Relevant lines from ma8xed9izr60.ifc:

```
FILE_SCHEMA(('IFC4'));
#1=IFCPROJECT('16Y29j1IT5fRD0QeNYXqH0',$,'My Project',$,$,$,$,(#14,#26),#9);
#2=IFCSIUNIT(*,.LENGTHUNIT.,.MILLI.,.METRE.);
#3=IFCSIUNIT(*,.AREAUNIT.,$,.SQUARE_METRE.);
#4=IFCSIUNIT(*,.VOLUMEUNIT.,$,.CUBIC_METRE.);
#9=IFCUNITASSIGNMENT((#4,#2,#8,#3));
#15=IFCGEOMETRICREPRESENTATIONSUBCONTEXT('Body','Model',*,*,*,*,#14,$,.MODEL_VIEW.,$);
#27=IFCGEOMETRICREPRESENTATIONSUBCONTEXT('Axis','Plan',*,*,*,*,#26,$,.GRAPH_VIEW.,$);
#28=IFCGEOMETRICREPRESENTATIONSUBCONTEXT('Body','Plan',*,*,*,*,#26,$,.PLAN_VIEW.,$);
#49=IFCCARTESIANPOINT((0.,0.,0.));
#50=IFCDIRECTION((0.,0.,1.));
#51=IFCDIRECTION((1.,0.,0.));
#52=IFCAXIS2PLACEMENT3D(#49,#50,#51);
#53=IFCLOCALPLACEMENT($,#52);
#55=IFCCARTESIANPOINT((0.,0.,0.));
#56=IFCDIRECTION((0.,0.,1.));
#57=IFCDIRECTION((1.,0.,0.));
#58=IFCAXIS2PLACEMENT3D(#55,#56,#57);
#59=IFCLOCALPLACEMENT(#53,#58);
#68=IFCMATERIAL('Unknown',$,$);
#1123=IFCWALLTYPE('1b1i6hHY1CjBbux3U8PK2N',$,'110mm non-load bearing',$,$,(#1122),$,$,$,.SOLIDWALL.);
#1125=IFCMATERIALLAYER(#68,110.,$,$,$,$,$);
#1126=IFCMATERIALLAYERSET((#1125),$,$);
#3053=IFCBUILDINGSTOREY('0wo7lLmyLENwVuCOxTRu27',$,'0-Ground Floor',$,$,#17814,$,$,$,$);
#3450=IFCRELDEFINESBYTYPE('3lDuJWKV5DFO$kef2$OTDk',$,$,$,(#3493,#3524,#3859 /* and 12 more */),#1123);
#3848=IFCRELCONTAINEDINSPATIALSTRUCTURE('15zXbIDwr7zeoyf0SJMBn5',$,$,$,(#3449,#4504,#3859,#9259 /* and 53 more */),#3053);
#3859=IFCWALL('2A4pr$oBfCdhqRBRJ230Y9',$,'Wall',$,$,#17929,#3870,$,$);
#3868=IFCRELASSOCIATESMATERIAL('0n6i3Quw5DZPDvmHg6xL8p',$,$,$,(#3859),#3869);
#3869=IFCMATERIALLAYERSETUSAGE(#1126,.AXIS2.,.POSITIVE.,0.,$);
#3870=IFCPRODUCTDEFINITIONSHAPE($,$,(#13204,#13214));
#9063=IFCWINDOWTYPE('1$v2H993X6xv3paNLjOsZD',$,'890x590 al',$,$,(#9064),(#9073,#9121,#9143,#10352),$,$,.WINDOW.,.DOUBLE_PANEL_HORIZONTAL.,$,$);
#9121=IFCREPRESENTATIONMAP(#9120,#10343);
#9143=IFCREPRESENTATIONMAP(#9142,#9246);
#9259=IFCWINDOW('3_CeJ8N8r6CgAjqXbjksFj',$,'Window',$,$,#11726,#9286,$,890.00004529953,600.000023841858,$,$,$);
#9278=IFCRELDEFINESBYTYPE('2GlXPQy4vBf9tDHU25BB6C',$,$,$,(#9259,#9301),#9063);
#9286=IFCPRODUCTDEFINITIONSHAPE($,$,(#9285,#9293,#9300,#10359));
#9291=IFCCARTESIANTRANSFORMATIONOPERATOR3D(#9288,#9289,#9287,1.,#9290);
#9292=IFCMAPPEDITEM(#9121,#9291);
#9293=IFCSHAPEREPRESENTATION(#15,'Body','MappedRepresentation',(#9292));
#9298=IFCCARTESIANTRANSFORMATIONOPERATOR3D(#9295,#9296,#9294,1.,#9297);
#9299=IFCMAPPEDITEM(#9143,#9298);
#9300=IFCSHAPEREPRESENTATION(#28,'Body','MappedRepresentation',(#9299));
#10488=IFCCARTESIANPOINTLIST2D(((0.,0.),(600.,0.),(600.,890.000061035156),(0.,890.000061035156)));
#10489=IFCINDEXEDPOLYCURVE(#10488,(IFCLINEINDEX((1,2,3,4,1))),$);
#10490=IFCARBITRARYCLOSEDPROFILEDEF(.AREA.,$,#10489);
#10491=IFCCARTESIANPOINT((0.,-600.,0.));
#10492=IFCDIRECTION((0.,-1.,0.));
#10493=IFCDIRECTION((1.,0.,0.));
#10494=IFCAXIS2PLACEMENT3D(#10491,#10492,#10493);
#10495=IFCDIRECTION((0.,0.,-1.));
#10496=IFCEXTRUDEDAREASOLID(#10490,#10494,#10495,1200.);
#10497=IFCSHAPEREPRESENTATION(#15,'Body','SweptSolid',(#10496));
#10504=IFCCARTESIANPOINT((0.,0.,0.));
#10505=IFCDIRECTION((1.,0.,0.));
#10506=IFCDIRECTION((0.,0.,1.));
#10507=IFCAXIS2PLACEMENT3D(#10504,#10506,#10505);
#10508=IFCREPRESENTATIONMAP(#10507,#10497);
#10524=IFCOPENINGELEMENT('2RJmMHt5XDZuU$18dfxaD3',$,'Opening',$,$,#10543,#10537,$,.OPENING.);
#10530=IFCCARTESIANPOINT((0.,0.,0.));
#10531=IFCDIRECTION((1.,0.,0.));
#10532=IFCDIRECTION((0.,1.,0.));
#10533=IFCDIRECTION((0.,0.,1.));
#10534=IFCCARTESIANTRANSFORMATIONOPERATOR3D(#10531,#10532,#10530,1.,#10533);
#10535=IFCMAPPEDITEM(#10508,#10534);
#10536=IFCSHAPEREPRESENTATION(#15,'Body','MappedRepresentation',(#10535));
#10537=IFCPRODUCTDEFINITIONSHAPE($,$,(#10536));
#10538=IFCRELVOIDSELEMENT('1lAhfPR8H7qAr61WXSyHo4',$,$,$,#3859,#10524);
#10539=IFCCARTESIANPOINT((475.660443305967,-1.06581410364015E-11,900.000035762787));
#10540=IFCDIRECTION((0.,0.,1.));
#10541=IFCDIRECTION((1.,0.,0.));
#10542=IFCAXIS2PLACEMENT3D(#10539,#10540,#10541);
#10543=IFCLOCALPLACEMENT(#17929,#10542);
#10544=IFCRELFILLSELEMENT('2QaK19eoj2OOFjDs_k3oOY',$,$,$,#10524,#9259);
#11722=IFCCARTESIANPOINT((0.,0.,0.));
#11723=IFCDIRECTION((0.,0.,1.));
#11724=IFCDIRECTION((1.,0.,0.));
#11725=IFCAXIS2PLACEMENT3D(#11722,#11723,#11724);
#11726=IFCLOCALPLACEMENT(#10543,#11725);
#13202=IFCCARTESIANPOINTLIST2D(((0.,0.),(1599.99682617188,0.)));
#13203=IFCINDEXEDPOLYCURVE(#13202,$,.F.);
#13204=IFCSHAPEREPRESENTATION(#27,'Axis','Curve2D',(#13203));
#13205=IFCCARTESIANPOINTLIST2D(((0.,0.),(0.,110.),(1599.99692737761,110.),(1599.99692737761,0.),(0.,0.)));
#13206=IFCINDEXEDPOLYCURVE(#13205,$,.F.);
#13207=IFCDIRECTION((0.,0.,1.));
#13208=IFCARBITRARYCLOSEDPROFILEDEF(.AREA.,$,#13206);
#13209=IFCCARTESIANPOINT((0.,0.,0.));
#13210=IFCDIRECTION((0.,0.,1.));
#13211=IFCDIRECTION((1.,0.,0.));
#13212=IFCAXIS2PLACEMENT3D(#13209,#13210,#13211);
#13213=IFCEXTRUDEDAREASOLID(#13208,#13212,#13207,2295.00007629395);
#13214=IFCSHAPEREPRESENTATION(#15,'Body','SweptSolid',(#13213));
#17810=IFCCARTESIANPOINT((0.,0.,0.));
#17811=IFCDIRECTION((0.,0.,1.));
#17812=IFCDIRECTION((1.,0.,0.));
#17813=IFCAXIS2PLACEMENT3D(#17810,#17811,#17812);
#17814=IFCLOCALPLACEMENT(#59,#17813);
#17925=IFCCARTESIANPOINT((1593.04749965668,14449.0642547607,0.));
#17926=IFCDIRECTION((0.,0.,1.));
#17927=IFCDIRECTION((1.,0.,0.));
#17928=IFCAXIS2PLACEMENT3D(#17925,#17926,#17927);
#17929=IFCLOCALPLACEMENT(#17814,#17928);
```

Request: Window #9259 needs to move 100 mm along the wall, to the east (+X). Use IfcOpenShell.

```python
import ifcopenshell
import ifcopenshell.api.geometry
import ifcopenshell.util.placement

model = ifcopenshell.open("ma8xed9izr60.ifc")

window = model.by_guid("3_CeJ8N8r6CgAjqXbjksFj")
opening = window.FillsVoids[0].RelatingOpeningElement
wall = opening.VoidsElements[0].RelatingBuildingElement

wall_matrix = ifcopenshell.util.placement.get_local_placement(wall.ObjectPlacement)
shift = wall_matrix[:3, 0] * 100.0
before = ifcopenshell.util.placement.get_local_placement(window.ObjectPlacement)[:3, 3].copy()

# The window is placed relative to its opening, so it follows when the opening moves.
matrix = ifcopenshell.util.placement.get_local_placement(opening.ObjectPlacement)
matrix[:3, 3] += shift
ifcopenshell.api.geometry.edit_object_placement(
    model, product=opening, matrix=matrix, is_si=False, should_transform_children=True
)

after = ifcopenshell.util.placement.get_local_placement(window.ObjectPlacement)[:3, 3]
print("window moved by", (after - before).round(3) + 0.0)

model.write("ma8xed9izr60-out.ifc")
```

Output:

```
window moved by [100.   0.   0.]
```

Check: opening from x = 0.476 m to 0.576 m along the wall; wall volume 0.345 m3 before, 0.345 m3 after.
